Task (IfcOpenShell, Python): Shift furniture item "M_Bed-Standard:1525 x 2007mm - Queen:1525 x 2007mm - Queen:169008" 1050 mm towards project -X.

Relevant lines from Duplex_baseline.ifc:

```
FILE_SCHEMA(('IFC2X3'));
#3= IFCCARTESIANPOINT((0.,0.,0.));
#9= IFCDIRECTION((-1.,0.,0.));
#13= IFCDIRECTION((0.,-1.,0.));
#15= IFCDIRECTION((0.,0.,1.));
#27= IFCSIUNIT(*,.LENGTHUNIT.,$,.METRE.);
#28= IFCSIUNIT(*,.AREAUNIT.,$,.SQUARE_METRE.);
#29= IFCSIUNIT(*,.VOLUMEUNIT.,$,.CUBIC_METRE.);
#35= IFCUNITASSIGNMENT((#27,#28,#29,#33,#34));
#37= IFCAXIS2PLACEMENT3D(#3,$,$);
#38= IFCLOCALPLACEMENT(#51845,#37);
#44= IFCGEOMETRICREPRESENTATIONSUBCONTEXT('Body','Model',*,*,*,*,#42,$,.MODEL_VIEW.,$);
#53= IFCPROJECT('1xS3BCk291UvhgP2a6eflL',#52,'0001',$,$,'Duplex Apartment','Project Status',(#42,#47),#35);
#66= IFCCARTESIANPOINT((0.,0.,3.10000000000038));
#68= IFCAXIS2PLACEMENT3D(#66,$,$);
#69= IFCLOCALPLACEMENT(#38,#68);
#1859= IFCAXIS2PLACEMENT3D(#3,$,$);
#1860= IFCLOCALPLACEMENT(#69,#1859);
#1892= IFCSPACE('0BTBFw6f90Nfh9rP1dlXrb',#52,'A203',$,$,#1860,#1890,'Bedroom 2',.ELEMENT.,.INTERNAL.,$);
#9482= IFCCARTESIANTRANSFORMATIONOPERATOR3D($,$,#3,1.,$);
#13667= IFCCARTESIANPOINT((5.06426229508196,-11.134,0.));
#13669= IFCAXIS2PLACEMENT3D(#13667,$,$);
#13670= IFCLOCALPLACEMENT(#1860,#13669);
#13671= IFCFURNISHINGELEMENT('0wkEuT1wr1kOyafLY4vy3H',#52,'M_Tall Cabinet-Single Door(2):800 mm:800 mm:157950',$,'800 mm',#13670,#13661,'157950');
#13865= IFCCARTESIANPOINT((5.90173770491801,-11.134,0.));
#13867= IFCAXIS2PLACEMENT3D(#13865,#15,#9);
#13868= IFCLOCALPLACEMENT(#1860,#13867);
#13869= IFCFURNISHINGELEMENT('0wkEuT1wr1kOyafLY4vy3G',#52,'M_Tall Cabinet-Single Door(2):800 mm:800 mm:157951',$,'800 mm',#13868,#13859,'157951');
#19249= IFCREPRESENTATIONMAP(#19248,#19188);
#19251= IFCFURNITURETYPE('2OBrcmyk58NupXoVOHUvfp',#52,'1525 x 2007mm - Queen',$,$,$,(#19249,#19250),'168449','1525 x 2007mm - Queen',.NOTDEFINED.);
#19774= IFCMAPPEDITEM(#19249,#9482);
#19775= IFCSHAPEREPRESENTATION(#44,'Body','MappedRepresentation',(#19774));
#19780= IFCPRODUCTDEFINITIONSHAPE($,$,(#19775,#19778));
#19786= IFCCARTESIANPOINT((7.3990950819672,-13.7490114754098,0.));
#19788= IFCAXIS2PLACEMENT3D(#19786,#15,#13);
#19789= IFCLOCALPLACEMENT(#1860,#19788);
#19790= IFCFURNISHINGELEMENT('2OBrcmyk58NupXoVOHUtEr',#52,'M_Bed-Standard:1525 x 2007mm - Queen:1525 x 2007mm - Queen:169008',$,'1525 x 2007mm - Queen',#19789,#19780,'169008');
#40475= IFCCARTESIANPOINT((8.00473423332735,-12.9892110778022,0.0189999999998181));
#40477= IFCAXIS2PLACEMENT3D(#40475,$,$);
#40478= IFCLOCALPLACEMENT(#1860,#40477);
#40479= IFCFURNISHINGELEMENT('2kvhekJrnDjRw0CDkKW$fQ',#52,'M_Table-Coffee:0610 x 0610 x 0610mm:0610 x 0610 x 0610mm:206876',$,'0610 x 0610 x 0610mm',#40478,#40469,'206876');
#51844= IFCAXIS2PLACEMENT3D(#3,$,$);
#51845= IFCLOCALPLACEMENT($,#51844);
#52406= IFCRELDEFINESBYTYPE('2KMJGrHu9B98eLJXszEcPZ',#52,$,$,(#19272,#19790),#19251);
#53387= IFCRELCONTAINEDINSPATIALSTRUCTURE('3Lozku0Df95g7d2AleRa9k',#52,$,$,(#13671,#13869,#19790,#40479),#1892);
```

```python
import ifcopenshell
import ifcopenshell.api.geometry
import ifcopenshell.util.placement
import ifcopenshell.util.unit

model = ifcopenshell.open("Duplex_baseline.ifc")
unit_scale = ifcopenshell.util.unit.calculate_unit_scale(model)

item = model.by_guid("2OBrcmyk58NupXoVOHUtEr")
matrix = ifcopenshell.util.placement.get_local_placement(item.ObjectPlacement)
matrix[0, 3] -= 1.05 / unit_scale
ifcopenshell.api.geometry.edit_object_placement(model, product=item, matrix=matrix, is_si=False)

print(ifcopenshell.util.placement.get_local_placement(item.ObjectPlacement).round(3) + 0.0)

model.write("Duplex_baseline_updated.ifc")
```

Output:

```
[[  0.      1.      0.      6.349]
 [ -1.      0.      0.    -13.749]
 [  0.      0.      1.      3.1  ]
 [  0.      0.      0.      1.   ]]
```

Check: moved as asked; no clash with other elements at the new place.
